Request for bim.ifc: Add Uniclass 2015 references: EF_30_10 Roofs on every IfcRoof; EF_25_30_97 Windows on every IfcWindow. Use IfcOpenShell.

First a look at what the model holds.

```python
import ifcopenshell

model = ifcopenshell.open("bim.ifc")
print(model.schema)
print("classifications:", [c.Name for c in model.by_type("IfcClassification")])
for ifc_class in ("IfcDoor", "IfcRoof", "IfcStair", "IfcWall", "IfcWindow"):
    print(ifc_class, len(model.by_type(ifc_class)))
```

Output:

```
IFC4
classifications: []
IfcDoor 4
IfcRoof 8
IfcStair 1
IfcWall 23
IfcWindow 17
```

```python
import ifcopenshell
import ifcopenshell.api.classification

model = ifcopenshell.open("bim.ifc")

system = ifcopenshell.api.classification.add_classification(model, classification="Uniclass 2015")

codes = {
    "IfcRoof": ("EF_30_10", "Roofs"),
    "IfcWindow": ("EF_25_30_97", "Windows"),
}
for ifc_class, (code, name) in codes.items():
    products = model.by_type(ifc_class)
    ifcopenshell.api.classification.add_reference(
        model, products=products, classification=system, identification=code, name=name
    )
    print(code, len(products))

model.write("bim_rev.ifc")
```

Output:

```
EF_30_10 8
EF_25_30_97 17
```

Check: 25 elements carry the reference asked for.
